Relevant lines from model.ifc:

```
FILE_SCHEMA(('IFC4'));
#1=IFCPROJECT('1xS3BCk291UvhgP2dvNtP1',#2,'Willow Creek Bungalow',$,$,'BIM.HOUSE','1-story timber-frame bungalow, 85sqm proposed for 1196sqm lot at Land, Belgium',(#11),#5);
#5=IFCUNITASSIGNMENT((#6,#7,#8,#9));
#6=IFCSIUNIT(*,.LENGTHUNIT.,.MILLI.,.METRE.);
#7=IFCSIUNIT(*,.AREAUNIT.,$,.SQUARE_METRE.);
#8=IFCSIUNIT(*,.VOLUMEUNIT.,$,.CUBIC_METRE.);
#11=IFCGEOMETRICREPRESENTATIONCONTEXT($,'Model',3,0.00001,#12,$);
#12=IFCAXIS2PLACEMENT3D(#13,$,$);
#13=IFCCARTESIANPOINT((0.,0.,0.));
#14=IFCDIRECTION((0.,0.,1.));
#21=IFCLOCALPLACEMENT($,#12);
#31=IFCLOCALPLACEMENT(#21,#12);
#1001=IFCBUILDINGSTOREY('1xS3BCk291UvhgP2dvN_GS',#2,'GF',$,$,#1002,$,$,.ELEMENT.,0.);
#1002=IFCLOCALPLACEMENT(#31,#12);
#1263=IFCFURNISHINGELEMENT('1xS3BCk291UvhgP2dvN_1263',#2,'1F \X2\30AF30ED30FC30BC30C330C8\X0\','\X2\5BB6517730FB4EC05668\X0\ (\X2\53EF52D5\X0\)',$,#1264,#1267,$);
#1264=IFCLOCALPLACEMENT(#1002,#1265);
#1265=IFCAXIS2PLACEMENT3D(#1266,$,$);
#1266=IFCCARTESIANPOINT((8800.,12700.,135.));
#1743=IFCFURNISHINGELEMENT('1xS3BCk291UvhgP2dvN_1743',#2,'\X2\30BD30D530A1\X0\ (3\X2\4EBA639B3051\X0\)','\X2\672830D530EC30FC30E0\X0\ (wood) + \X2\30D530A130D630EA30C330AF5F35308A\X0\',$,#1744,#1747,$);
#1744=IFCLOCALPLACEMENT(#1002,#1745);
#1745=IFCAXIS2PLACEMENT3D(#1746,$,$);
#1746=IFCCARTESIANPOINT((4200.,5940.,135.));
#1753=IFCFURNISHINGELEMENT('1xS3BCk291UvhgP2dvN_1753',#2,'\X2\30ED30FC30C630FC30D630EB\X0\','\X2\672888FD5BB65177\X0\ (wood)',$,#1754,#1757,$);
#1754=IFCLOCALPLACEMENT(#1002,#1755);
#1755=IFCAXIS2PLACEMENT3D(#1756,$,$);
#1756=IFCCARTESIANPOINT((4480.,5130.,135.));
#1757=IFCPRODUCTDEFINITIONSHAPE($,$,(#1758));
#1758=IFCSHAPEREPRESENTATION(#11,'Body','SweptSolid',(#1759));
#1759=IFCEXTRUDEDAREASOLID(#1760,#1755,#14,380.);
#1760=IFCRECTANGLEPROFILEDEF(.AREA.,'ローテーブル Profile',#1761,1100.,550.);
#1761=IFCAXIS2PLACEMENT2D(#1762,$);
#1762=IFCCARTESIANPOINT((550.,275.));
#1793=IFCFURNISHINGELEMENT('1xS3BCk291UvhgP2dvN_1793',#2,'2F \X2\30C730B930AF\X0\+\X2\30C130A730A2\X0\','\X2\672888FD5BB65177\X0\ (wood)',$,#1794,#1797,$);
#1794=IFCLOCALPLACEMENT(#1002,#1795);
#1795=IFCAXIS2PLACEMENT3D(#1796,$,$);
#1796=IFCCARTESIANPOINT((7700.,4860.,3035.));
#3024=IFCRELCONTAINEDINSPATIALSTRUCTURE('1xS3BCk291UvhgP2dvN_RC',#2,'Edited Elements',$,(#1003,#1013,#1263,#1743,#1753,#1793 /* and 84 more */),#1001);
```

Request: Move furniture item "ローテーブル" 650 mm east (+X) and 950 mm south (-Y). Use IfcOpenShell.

```python
import ifcopenshell
import ifcopenshell.api.geometry
import ifcopenshell.util.placement

model = ifcopenshell.open("model.ifc")

item = model.by_guid("1xS3BCk291UvhgP2dvN_1753")
matrix = ifcopenshell.util.placement.get_local_placement(item.ObjectPlacement)
matrix[0, 3] += 650.0
matrix[1, 3] -= 950.0
ifcopenshell.api.geometry.edit_object_placement(model, product=item, matrix=matrix, is_si=False)

print(ifcopenshell.util.placement.get_local_placement(item.ObjectPlacement).round(3) + 0.0)

model.write("model_rev.ifc")
```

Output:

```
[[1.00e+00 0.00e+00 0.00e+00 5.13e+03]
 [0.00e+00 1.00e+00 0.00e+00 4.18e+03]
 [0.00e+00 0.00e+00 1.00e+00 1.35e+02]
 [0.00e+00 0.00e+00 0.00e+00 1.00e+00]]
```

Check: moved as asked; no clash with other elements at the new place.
